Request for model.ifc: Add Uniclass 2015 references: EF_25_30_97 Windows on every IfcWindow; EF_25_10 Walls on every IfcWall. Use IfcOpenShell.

First a look at what the model holds.

```python
import ifcopenshell

model = ifcopenshell.open("model.ifc")
print(model.schema)
print("classifications:", [c.Name for c in model.by_type("IfcClassification")])
for ifc_class in ("IfcDoor", "IfcRoof", "IfcStair", "IfcWall", "IfcWindow"):
    print(ifc_class, len(model.by_type(ifc_class)))
```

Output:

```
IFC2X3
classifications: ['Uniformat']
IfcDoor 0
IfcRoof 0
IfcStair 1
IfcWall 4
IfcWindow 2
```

```python
import ifcopenshell
import ifcopenshell.api.classification

model = ifcopenshell.open("model.ifc")

# IFC2X3 requires Source and Edition and has no link from the project to the system.
system = model.create_entity("IfcClassification", Source="NBS", Edition="2015", Name="Uniclass 2015")

codes = {
    "IfcWindow": ("EF_25_30_97", "Windows"),
    "IfcWall": ("EF_25_10", "Walls"),
}
for ifc_class, (code, name) in codes.items():
    products = model.by_type(ifc_class)
    ifcopenshell.api.classification.add_reference(
        model, products=products, classification=system, identification=code, name=name
    )
    print(code, len(products))

model.write("model_updated.ifc")
```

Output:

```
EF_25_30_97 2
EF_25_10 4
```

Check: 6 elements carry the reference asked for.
